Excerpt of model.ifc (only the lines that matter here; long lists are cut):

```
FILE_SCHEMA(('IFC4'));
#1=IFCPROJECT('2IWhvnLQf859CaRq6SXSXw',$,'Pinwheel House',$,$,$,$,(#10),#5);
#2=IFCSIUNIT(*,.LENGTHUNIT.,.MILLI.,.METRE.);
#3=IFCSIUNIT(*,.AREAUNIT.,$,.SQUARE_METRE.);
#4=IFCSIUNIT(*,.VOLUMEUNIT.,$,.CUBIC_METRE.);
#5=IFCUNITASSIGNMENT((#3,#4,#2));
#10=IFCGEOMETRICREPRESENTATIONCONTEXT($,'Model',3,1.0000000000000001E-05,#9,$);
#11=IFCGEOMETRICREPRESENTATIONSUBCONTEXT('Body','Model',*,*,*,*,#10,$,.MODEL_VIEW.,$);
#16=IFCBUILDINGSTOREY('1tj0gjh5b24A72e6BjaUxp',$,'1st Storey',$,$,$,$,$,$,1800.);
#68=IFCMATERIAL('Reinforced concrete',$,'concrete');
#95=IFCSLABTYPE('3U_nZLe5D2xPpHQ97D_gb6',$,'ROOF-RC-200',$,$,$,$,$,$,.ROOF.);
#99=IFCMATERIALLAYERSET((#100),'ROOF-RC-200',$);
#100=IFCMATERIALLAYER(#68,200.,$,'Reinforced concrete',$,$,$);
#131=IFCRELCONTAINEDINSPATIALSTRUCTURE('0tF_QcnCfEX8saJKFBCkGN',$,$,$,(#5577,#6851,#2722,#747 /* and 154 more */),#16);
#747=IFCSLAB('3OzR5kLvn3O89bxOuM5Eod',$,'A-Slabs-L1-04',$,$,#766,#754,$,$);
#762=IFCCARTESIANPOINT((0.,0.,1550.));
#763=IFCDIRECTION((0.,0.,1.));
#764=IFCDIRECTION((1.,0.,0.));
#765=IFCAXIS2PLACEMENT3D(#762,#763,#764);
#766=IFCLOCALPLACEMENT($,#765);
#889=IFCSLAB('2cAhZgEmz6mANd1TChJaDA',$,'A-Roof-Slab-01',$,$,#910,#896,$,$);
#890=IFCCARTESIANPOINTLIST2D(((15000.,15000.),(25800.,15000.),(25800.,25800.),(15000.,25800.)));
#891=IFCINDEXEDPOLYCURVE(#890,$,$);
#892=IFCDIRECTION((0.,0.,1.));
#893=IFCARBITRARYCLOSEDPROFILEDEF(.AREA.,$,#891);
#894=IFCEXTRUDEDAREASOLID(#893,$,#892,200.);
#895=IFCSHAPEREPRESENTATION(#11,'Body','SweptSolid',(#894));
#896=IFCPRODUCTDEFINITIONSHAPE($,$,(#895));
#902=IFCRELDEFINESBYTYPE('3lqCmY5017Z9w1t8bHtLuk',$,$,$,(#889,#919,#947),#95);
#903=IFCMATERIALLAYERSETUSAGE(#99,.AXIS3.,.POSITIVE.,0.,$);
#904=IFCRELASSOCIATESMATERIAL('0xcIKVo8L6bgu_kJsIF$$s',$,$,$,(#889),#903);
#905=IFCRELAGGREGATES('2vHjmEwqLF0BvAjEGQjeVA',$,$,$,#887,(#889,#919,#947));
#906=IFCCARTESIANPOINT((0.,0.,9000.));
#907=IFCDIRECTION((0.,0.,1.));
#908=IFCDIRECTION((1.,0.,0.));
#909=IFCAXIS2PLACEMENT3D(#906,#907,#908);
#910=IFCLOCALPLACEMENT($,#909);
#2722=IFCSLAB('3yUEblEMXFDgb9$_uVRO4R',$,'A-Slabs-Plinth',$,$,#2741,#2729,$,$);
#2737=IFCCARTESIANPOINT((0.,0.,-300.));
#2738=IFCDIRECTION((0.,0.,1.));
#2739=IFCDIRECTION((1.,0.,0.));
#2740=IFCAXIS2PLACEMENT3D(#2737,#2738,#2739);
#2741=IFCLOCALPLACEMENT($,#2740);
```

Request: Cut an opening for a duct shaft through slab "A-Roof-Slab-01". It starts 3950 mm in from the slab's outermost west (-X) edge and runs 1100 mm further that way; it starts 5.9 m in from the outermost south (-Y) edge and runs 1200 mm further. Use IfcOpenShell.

```python
import numpy as np
import ifcopenshell
import ifcopenshell.api.feature
import ifcopenshell.api.geometry
import ifcopenshell.api.root
import ifcopenshell.geom
import ifcopenshell.util.placement
import ifcopenshell.util.representation
import ifcopenshell.util.shape
import ifcopenshell.util.unit

model = ifcopenshell.open("model.ifc")
unit_scale = ifcopenshell.util.unit.calculate_unit_scale(model)
settings = ifcopenshell.geom.settings()


def volume(element):
    """Net volume in cubic metres, openings subtracted."""
    shape = ifcopenshell.geom.create_shape(settings, element)
    return ifcopenshell.util.shape.get_volume(shape.geometry)


slab = model.by_guid("2cAhZgEmz6mANd1TChJaDA")
before = volume(slab)

# Extent in the slab's own axes, in metres. The edges named are its -X and -Y sides.
slab_shape = ifcopenshell.geom.create_shape(settings, slab)
vertices = ifcopenshell.util.shape.get_vertices(slab_shape.geometry)
x_min, y_min, bottom = vertices.min(axis=0)
top = vertices[:, 2].max()

opening = ifcopenshell.api.root.create_entity(model, ifc_class="IfcOpeningElement", name="Duct shaft opening", predefined_type="OPENING")
context = ifcopenshell.util.representation.get_context(model, "Model", "Body", "MODEL_VIEW")
width, depth = 1.1, 1.2
outline = [(0.0, 0.0), (width, 0.0), (width, depth), (0.0, depth), (0.0, 0.0)]
# Overshoot both faces by 50 mm so the cut is clean.
shape = ifcopenshell.api.geometry.add_slab_representation(
    model, context=context, depth=top - bottom + 0.1, polyline=outline
)
ifcopenshell.api.geometry.assign_representation(model, product=opening, representation=shape)

matrix = ifcopenshell.util.placement.get_local_placement(slab.ObjectPlacement)
matrix[:, 3] = matrix @ np.append(np.array([x_min + 3.95, y_min + 5.9, bottom - 0.05]) / unit_scale, 1.0)
ifcopenshell.api.geometry.edit_object_placement(model, product=opening, matrix=matrix, is_si=False)
ifcopenshell.api.feature.add_feature(model, feature=opening, element=slab)

after = volume(slab)

print(f"slab volume {before:.3f} -> {after:.3f} m3")

model.write("model_edited.ifc")
```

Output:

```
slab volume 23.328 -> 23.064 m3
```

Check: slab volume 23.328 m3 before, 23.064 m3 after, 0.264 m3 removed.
